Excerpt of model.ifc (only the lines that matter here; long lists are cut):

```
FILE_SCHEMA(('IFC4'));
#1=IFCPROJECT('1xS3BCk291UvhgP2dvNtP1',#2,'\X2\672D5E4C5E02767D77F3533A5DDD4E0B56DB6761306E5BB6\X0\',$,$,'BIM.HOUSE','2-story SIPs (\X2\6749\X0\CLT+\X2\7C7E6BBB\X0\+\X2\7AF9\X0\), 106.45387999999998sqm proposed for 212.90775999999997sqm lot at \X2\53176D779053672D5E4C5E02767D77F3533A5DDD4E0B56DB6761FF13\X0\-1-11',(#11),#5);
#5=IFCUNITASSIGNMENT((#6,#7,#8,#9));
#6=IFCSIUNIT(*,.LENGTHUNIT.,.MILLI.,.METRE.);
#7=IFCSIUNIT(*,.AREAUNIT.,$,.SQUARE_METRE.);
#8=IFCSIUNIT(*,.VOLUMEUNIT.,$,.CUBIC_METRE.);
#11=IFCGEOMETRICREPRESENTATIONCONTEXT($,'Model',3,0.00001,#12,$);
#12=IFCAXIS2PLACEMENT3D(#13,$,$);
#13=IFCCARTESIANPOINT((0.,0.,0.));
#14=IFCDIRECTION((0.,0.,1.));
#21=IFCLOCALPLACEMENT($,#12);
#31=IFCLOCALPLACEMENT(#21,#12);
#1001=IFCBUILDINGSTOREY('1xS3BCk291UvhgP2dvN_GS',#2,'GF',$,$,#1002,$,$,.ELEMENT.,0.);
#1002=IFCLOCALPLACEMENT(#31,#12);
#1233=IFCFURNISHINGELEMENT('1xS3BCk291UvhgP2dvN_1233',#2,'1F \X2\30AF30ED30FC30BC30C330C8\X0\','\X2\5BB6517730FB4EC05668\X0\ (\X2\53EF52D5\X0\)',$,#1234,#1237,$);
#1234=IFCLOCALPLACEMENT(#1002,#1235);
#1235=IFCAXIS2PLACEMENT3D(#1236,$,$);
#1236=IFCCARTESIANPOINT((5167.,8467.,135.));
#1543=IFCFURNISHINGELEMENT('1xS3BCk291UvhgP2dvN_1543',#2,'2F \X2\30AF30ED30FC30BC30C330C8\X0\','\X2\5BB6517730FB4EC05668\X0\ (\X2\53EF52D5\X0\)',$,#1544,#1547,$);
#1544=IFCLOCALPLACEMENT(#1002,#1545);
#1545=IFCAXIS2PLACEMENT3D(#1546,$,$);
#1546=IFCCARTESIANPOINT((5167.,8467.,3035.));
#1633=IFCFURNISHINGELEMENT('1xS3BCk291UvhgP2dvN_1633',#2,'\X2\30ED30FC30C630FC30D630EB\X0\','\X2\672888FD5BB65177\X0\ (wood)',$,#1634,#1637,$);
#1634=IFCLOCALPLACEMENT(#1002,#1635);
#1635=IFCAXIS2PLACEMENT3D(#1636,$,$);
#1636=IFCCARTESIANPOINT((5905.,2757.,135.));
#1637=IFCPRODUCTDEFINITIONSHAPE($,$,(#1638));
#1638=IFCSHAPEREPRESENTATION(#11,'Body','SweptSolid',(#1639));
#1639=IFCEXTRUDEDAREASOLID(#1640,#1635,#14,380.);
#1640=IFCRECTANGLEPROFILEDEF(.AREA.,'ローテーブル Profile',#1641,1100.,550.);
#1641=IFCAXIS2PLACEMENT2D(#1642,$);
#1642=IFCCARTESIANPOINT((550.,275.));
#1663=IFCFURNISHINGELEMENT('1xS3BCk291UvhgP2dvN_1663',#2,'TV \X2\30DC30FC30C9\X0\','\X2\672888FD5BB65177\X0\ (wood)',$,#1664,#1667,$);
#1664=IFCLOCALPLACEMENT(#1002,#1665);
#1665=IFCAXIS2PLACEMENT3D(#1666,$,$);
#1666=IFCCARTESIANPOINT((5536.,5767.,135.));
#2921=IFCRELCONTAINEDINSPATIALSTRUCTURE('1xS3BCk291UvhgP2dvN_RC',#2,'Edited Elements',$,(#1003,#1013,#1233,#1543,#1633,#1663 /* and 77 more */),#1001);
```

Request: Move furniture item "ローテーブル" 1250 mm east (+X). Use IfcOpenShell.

```python
import ifcopenshell
import ifcopenshell.api.geometry
import ifcopenshell.util.placement

model = ifcopenshell.open("model.ifc")

item = model.by_guid("1xS3BCk291UvhgP2dvN_1633")
matrix = ifcopenshell.util.placement.get_local_placement(item.ObjectPlacement)
matrix[0, 3] += 1250.0
ifcopenshell.api.geometry.edit_object_placement(model, product=item, matrix=matrix, is_si=False)

print(ifcopenshell.util.placement.get_local_placement(item.ObjectPlacement).round(3) + 0.0)

model.write("model_v2.ifc")
```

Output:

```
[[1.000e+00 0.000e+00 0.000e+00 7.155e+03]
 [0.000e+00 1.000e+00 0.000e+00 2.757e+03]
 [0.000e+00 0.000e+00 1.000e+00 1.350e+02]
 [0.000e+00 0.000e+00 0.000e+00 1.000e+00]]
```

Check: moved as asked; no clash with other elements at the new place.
